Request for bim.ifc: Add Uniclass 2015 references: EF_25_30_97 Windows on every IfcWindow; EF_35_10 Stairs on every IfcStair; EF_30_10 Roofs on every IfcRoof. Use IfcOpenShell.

First a look at what the model holds.

```python
import ifcopenshell

model = ifcopenshell.open("bim.ifc")
print(model.schema)
print("classifications:", [c.Name for c in model.by_type("IfcClassification")])
for ifc_class in ("IfcDoor", "IfcRoof", "IfcStair", "IfcWall", "IfcWindow"):
    print(ifc_class, len(model.by_type(ifc_class)))
```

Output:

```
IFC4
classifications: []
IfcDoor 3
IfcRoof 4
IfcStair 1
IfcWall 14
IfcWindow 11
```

```python
import ifcopenshell
import ifcopenshell.api.classification

model = ifcopenshell.open("bim.ifc")

system = ifcopenshell.api.classification.add_classification(model, classification="Uniclass 2015")

codes = {
    "IfcWindow": ("EF_25_30_97", "Windows"),
    "IfcStair": ("EF_35_10", "Stairs"),
    "IfcRoof": ("EF_30_10", "Roofs"),
}
for ifc_class, (code, name) in codes.items():
    products = model.by_type(ifc_class)
    ifcopenshell.api.classification.add_reference(
        model, products=products, classification=system, identification=code, name=name
    )
    print(code, len(products))

model.write("bim_edited.ifc")
```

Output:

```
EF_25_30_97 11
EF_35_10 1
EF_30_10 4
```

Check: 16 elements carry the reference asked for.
